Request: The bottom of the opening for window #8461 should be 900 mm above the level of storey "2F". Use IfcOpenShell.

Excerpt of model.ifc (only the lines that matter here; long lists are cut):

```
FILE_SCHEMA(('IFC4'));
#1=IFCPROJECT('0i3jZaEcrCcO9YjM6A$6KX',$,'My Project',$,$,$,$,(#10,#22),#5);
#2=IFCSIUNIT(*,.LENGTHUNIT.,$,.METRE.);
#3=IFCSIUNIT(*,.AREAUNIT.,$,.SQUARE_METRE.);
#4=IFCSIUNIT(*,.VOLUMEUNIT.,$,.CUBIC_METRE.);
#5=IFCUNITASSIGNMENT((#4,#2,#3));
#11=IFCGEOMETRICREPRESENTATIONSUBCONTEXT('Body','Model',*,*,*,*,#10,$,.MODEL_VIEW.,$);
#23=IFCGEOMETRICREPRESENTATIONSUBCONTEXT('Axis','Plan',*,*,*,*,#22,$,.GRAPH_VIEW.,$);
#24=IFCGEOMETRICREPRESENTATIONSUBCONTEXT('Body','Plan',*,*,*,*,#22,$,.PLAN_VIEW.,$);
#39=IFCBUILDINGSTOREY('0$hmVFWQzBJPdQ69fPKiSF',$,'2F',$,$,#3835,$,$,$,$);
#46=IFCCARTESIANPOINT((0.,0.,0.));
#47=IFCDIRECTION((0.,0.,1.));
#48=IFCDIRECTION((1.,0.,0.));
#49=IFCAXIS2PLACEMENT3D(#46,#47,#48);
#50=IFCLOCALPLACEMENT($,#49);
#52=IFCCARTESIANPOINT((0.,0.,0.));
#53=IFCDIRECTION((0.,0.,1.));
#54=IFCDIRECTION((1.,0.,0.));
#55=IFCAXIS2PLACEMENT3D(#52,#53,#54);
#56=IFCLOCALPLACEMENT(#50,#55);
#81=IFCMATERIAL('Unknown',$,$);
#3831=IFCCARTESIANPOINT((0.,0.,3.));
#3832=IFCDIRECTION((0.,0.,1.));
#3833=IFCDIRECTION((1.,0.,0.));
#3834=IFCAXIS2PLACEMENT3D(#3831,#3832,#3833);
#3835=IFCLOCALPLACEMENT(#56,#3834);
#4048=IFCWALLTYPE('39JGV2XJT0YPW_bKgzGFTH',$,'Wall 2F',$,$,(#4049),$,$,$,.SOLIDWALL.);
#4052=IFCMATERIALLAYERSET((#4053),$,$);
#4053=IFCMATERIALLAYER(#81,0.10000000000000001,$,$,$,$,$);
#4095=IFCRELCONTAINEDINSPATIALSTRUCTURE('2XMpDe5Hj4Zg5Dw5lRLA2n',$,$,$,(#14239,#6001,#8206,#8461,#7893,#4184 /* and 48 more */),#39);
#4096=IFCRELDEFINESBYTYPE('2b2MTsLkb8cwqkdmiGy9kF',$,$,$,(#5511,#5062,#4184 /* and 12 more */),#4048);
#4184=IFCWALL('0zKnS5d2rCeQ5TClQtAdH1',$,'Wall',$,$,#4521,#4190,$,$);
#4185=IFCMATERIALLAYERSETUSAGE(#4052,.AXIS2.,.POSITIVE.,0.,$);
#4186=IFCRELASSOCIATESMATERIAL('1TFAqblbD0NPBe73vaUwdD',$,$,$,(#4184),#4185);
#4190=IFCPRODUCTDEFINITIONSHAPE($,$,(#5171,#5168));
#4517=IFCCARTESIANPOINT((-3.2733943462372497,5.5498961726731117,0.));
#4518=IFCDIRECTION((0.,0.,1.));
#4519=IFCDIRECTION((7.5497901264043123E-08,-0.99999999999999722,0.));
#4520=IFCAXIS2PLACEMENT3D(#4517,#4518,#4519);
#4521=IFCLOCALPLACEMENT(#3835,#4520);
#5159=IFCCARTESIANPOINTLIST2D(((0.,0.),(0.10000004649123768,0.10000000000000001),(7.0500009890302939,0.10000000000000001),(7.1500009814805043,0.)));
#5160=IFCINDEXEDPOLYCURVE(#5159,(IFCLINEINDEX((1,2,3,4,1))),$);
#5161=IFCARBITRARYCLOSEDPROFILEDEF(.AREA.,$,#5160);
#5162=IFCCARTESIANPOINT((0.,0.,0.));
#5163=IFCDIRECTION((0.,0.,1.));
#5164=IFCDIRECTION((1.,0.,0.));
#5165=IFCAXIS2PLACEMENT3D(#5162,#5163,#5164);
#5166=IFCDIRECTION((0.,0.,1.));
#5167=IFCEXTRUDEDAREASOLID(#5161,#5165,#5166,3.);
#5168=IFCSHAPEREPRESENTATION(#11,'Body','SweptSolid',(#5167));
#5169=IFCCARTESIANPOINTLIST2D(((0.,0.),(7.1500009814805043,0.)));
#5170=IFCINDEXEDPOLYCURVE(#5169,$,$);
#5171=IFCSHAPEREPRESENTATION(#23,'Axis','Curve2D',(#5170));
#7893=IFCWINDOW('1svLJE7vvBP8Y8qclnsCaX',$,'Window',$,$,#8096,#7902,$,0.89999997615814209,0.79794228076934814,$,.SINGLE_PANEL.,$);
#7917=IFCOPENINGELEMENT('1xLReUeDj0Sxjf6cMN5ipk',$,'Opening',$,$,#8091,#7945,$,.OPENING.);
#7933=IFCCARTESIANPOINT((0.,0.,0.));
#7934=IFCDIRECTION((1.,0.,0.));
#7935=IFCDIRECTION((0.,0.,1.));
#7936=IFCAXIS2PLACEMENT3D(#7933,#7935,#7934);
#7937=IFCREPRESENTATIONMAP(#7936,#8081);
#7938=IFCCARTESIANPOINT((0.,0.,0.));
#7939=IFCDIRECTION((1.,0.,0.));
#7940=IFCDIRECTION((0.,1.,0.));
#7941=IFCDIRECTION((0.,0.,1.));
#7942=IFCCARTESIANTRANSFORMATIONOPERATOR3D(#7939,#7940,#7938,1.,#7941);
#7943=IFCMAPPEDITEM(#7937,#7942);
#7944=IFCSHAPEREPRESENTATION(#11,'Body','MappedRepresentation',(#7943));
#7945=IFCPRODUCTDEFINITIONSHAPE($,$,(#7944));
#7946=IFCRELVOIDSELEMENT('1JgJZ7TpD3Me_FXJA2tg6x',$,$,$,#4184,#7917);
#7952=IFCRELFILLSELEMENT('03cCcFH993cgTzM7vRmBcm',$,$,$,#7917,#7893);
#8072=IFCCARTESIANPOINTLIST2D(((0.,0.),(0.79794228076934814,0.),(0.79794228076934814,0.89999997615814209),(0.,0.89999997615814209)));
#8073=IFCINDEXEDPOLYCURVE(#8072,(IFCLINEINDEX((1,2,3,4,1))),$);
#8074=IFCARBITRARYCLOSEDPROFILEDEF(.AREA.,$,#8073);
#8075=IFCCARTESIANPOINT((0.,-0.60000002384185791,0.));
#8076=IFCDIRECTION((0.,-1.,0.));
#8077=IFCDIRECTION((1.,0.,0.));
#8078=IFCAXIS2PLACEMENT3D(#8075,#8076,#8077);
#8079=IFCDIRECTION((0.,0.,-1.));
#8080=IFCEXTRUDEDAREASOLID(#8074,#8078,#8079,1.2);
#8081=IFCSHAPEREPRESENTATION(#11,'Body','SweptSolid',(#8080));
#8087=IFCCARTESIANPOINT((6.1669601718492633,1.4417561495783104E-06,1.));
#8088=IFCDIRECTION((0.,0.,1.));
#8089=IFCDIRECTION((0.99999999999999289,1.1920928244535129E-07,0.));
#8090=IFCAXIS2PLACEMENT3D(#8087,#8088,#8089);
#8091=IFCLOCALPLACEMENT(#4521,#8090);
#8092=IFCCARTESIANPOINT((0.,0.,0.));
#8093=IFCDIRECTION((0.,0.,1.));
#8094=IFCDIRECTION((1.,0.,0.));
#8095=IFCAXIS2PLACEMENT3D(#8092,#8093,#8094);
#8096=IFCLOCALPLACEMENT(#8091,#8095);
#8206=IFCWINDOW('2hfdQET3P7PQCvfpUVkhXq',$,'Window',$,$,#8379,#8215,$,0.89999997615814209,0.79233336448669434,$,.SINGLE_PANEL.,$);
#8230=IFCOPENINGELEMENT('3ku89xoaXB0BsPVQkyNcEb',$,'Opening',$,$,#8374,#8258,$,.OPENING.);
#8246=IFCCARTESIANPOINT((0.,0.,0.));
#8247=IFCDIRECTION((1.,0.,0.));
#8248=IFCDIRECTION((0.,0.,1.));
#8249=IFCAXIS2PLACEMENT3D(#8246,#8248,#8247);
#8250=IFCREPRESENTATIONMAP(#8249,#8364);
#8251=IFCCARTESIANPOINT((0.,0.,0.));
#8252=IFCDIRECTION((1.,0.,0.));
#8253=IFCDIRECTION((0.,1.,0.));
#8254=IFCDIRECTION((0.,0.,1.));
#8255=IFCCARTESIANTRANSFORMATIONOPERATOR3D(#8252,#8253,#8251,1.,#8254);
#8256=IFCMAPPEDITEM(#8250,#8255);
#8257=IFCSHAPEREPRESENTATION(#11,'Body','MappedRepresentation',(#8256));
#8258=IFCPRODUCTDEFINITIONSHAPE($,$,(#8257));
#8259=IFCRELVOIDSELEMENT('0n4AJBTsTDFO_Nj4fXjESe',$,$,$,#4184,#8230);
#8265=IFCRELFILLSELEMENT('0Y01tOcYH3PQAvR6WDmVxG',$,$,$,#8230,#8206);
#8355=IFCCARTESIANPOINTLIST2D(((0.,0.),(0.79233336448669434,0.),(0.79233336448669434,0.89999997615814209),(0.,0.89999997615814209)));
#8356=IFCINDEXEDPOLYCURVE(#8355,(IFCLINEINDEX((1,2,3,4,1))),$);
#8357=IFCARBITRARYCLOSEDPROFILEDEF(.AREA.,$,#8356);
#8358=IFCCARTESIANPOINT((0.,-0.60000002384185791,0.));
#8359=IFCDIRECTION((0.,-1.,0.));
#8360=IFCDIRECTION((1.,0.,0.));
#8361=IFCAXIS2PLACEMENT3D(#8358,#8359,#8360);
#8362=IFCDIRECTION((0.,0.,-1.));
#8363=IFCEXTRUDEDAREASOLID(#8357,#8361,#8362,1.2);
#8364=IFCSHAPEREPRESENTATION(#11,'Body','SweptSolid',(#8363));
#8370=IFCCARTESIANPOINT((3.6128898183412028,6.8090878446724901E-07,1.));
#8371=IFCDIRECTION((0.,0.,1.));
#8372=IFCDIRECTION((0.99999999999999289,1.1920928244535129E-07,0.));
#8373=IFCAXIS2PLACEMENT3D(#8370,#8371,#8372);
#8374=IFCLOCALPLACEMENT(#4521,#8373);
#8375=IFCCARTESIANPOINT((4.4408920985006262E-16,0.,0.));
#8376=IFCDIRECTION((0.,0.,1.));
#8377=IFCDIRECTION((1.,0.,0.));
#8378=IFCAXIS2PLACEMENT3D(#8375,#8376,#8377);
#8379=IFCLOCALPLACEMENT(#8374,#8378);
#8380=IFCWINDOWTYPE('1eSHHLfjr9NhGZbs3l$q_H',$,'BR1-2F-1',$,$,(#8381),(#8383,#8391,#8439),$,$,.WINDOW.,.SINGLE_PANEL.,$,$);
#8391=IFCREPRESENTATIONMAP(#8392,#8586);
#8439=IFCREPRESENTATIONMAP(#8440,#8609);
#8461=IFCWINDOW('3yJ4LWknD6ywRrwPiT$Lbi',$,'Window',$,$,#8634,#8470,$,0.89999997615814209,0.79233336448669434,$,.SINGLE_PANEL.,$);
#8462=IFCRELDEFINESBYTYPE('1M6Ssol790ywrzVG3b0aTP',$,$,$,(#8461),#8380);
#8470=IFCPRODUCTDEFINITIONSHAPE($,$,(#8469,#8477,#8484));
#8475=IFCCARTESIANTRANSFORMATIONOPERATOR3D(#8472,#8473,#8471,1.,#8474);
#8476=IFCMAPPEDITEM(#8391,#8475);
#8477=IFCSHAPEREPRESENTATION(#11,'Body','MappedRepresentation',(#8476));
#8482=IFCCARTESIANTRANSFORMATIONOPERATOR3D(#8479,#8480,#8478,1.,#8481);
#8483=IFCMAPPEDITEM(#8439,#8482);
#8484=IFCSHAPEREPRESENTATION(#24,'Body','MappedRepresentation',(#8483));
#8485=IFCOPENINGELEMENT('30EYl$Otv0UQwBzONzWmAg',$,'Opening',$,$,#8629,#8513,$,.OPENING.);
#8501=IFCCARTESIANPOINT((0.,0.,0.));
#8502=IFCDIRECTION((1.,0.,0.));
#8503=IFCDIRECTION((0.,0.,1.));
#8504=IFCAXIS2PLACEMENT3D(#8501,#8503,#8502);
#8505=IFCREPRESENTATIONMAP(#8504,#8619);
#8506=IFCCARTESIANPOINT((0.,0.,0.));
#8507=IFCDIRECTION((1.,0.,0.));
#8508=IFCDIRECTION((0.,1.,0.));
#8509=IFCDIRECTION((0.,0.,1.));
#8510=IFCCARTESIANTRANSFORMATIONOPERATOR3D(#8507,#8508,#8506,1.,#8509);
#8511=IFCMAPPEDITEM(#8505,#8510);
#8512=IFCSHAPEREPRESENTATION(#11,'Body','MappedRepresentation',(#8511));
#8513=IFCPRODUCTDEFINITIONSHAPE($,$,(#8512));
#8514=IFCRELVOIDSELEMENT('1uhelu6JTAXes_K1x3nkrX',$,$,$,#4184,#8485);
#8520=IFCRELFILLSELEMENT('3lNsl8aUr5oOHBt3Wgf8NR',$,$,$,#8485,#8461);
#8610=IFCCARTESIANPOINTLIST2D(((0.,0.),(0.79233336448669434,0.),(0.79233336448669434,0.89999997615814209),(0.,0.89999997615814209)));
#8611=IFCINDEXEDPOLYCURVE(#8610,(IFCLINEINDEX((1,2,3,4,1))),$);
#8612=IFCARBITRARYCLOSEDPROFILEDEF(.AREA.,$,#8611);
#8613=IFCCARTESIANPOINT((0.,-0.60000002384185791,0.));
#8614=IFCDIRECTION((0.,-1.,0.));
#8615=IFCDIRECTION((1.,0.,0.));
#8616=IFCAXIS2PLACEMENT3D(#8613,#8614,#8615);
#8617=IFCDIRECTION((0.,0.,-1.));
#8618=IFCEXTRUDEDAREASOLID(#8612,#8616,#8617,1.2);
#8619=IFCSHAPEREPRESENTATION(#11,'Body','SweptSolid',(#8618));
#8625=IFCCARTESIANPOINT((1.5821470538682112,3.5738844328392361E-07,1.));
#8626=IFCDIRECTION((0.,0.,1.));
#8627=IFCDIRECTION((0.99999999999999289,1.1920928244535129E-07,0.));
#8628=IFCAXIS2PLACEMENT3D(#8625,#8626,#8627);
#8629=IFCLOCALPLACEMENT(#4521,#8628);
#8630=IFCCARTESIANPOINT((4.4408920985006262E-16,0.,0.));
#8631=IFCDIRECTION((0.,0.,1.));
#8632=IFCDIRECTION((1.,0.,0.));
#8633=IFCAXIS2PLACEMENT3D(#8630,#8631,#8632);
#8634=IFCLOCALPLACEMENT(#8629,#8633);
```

```python
import numpy as np
import ifcopenshell
import ifcopenshell.api.geometry
import ifcopenshell.geom
import ifcopenshell.util.element
import ifcopenshell.util.placement
import ifcopenshell.util.shape
import ifcopenshell.util.unit

model = ifcopenshell.open("model.ifc")
unit_scale = ifcopenshell.util.unit.calculate_unit_scale(model)

window = model.by_guid("3yJ4LWknD6ywRrwPiT$Lbi")
opening = window.FillsVoids[0].RelatingOpeningElement
storey = ifcopenshell.util.element.get_container(window, ifc_class="IfcBuildingStorey")
level = ifcopenshell.util.placement.get_local_placement(storey.ObjectPlacement)[2, 3]

# The opening's origin need not be at the sill, so measure its lowest point.
shape = ifcopenshell.geom.create_shape(ifcopenshell.geom.settings(), opening)
bottom = ifcopenshell.util.shape.get_shape_bottom_elevation(shape, shape.geometry) / unit_scale
dz = level + 0.9 - bottom

shift = np.array([0.0, 0.0, dz])
# The window is placed relative to its opening, so it follows when the opening moves.
matrix = ifcopenshell.util.placement.get_local_placement(opening.ObjectPlacement)
matrix[:3, 3] += shift
ifcopenshell.api.geometry.edit_object_placement(
    model, product=opening, matrix=matrix, is_si=False, should_transform_children=True
)

print(f"moved by {dz * unit_scale:+.3f} m")

model.write("model_edited.ifc")
```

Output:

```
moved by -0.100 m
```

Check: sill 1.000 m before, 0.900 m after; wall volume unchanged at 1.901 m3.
